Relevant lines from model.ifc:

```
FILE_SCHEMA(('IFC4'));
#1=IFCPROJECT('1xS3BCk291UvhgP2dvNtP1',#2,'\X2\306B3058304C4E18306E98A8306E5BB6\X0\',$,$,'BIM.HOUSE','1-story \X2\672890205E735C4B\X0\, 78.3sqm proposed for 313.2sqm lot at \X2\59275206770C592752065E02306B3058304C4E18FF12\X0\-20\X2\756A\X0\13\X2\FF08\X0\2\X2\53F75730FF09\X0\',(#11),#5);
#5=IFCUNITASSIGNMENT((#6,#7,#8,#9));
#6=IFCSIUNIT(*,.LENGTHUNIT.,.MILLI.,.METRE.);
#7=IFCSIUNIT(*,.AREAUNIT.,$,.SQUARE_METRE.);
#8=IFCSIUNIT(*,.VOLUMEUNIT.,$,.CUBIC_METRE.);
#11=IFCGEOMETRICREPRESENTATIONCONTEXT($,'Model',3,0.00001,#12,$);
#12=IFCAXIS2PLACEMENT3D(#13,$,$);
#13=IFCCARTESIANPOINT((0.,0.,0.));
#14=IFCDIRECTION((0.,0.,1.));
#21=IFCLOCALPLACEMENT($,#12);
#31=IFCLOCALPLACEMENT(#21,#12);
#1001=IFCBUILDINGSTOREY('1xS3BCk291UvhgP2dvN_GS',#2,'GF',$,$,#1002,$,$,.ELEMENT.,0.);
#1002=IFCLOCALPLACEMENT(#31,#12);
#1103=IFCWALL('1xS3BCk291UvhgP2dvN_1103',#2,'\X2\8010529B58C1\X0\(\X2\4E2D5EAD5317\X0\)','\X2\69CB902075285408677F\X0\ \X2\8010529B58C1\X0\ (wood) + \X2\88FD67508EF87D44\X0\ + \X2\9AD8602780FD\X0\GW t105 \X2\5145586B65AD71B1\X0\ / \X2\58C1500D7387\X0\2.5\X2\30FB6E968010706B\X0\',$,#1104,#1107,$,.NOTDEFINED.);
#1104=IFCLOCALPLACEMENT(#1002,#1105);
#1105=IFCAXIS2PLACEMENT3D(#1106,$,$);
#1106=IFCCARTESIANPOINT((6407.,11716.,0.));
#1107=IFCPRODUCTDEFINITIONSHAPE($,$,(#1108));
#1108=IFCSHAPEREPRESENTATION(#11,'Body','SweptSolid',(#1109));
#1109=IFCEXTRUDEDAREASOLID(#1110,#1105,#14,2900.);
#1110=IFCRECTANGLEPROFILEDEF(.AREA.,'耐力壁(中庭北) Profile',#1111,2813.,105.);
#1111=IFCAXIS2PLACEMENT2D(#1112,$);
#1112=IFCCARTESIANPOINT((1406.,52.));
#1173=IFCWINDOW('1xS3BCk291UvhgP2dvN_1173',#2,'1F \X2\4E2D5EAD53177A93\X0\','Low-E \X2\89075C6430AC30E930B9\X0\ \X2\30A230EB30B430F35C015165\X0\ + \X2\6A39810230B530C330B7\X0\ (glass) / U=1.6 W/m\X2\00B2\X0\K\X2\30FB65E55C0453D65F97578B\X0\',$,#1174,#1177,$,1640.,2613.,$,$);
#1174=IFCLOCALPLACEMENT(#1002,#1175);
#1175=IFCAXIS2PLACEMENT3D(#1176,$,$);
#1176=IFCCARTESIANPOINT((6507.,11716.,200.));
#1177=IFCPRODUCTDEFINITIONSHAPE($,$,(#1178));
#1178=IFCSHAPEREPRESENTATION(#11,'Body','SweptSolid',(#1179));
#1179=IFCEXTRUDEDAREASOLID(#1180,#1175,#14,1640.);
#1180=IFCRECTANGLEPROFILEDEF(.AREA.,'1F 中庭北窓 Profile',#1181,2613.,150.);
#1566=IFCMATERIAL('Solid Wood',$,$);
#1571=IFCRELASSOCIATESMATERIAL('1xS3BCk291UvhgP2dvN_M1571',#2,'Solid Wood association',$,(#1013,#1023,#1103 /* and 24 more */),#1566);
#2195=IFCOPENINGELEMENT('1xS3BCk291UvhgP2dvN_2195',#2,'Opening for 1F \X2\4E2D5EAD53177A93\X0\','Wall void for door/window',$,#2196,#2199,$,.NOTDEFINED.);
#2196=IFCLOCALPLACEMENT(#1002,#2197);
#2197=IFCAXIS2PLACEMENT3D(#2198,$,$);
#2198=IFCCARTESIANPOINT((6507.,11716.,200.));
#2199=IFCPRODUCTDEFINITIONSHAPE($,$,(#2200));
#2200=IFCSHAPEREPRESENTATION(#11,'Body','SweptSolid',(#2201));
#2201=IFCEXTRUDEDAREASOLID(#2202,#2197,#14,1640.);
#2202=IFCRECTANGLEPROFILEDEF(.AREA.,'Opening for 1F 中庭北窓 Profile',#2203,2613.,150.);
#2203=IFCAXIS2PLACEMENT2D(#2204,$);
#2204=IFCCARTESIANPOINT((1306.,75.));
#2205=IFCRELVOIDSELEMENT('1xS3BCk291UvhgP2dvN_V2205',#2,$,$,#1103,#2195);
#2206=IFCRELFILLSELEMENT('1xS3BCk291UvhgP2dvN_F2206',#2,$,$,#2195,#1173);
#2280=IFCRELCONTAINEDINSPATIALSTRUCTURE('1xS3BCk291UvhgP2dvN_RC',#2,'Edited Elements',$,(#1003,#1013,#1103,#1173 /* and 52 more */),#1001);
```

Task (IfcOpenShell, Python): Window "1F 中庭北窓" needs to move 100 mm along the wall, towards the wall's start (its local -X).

```python
import ifcopenshell
import ifcopenshell.api.geometry
import ifcopenshell.util.placement
import ifcopenshell.util.unit

model = ifcopenshell.open("model.ifc")
unit_scale = ifcopenshell.util.unit.calculate_unit_scale(model)

window = model.by_guid("1xS3BCk291UvhgP2dvN_1173")
opening = window.FillsVoids[0].RelatingOpeningElement
wall = opening.VoidsElements[0].RelatingBuildingElement

wall_matrix = ifcopenshell.util.placement.get_local_placement(wall.ObjectPlacement)
shift = wall_matrix[:3, 0] * -0.1 / unit_scale
before = ifcopenshell.util.placement.get_local_placement(window.ObjectPlacement)[:3, 3].copy()

# The window is not placed relative to its opening, so move both.
for product in (opening, window):
    matrix = ifcopenshell.util.placement.get_local_placement(product.ObjectPlacement)
    matrix[:3, 3] += shift
    ifcopenshell.api.geometry.edit_object_placement(model, product=product, matrix=matrix, is_si=False)

after = ifcopenshell.util.placement.get_local_placement(window.ObjectPlacement)[:3, 3]
print("window moved by", (after - before).round(3) + 0.0)

model.write("model_updated.ifc")
```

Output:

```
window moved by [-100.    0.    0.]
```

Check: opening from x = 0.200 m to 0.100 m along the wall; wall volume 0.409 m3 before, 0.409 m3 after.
